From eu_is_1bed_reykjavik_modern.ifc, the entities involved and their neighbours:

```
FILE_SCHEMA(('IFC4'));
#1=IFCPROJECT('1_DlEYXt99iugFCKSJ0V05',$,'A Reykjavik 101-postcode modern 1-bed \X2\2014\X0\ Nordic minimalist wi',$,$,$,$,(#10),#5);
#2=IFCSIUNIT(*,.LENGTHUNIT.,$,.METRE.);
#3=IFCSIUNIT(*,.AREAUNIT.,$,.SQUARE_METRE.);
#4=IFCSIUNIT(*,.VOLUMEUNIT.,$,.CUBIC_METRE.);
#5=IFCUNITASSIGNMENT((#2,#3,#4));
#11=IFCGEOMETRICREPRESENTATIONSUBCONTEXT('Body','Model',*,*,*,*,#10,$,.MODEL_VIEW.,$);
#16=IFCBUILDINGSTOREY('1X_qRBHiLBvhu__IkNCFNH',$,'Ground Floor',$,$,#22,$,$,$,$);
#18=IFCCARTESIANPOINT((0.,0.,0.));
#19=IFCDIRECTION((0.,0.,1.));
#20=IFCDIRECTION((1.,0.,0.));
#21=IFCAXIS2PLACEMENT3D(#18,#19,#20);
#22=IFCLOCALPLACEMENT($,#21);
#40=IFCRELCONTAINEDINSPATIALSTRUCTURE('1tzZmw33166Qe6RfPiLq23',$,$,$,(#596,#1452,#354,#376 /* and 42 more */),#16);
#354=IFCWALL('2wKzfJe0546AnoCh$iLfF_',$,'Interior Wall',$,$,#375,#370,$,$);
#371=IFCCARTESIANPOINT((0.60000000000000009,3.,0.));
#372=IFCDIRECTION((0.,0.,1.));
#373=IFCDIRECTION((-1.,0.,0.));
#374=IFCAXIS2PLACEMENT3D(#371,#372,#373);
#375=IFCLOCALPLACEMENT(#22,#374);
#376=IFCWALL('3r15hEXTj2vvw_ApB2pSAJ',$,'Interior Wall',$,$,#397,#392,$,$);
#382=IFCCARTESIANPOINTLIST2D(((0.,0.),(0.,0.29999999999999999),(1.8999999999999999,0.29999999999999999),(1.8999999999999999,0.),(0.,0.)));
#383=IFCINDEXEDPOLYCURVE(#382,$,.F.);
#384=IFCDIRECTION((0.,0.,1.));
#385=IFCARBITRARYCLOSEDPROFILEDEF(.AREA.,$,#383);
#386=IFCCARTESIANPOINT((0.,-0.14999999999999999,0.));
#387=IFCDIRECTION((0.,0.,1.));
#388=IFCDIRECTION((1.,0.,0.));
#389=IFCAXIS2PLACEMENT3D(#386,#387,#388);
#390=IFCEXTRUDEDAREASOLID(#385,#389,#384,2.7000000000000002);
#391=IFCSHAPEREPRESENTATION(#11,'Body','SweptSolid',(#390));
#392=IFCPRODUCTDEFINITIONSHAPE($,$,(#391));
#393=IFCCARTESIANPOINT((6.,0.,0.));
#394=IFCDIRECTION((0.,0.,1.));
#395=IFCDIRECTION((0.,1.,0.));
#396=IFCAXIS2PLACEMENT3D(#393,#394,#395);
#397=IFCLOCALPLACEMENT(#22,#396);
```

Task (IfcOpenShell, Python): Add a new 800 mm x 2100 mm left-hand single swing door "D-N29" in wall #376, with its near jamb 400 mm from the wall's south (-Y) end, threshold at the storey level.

```python
import numpy as np
import ifcopenshell
import ifcopenshell.api.feature
import ifcopenshell.api.geometry
import ifcopenshell.api.root
import ifcopenshell.api.spatial
import ifcopenshell.geom
import ifcopenshell.util.element
import ifcopenshell.util.placement
import ifcopenshell.util.representation
import ifcopenshell.util.shape
import ifcopenshell.util.unit

model = ifcopenshell.open("eu_is_1bed_reykjavik_modern.ifc")
unit_scale = ifcopenshell.util.unit.calculate_unit_scale(model)
settings = ifcopenshell.geom.settings()


def volume(element):
    """Net volume in cubic metres, openings subtracted."""
    shape = ifcopenshell.geom.create_shape(settings, element)
    return ifcopenshell.util.shape.get_volume(shape.geometry)


wall = model.by_guid("3r15hEXTj2vvw_ApB2pSAJ")
storey = ifcopenshell.util.element.get_container(wall, ifc_class="IfcBuildingStorey")
context = ifcopenshell.util.representation.get_context(model, "Model", "Body", "MODEL_VIEW")
before = volume(wall)

width, height, from_end, sill = 0.8, 2.1, 0.4, 0.0  # metres

# The wall runs along its own X axis, and the end named is its -X end.
wall_shape = ifcopenshell.geom.create_shape(settings, wall)
x, y, z = ifcopenshell.util.shape.get_vertices(wall_shape.geometry).T
start = x.min() + from_end
face, thickness = float(y.min()), float(y.max() - y.min())
wall_matrix = ifcopenshell.util.placement.get_local_placement(wall.ObjectPlacement)
level = ifcopenshell.util.placement.get_local_placement(storey.ObjectPlacement)[2, 3]


def in_wall(x, y):
    """Placement at x, y metres in the wall's axes, at sill height."""
    matrix = wall_matrix.copy()
    matrix[:, 3] = wall_matrix @ np.array([x / unit_scale, y / unit_scale, 0.0, 1.0])
    matrix[2, 3] = level + sill / unit_scale
    return matrix


# Opening: a box that overshoots both wall faces by 50 mm.
opening = ifcopenshell.api.root.create_entity(model, ifc_class="IfcOpeningElement", predefined_type="OPENING")
box = ifcopenshell.api.geometry.add_wall_representation(
    model, context=context, length=width, height=height, thickness=thickness + 0.1
)
ifcopenshell.api.geometry.assign_representation(model, product=opening, representation=box)
ifcopenshell.api.geometry.edit_object_placement(model, product=opening, matrix=in_wall(start, face - 0.05), is_si=False)
ifcopenshell.api.feature.add_feature(model, feature=opening, element=wall)

door = ifcopenshell.api.root.create_entity(model, ifc_class="IfcDoor", name="D-N29", predefined_type="DOOR")
door.OverallWidth, door.OverallHeight = width / unit_scale, height / unit_scale
door.OperationType = "SINGLE_SWING_LEFT"
body = ifcopenshell.api.geometry.add_door_representation(
    model,
    context=context,
    overall_width=door.OverallWidth,
    overall_height=door.OverallHeight,
    operation_type="SINGLE_SWING_LEFT",
    lining_properties={"LiningDepth": thickness / unit_scale, "ThresholdDepth": thickness / unit_scale},
)
ifcopenshell.api.geometry.assign_representation(model, product=door, representation=body)
ifcopenshell.api.spatial.assign_container(model, products=[door], relating_structure=storey)
ifcopenshell.api.feature.add_filling(model, opening=opening, element=door)

# The lining spans the wall, so the door starts at the wall face.
ifcopenshell.api.geometry.edit_object_placement(model, product=door, matrix=in_wall(start, face), is_si=False)

after = volume(wall)

print(f"wall volume {before:.3f} -> {after:.3f} m3")

model.write("eu_is_1bed_reykjavik_modern-out.ifc")
```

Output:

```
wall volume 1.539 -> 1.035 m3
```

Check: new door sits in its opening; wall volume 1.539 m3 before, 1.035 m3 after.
